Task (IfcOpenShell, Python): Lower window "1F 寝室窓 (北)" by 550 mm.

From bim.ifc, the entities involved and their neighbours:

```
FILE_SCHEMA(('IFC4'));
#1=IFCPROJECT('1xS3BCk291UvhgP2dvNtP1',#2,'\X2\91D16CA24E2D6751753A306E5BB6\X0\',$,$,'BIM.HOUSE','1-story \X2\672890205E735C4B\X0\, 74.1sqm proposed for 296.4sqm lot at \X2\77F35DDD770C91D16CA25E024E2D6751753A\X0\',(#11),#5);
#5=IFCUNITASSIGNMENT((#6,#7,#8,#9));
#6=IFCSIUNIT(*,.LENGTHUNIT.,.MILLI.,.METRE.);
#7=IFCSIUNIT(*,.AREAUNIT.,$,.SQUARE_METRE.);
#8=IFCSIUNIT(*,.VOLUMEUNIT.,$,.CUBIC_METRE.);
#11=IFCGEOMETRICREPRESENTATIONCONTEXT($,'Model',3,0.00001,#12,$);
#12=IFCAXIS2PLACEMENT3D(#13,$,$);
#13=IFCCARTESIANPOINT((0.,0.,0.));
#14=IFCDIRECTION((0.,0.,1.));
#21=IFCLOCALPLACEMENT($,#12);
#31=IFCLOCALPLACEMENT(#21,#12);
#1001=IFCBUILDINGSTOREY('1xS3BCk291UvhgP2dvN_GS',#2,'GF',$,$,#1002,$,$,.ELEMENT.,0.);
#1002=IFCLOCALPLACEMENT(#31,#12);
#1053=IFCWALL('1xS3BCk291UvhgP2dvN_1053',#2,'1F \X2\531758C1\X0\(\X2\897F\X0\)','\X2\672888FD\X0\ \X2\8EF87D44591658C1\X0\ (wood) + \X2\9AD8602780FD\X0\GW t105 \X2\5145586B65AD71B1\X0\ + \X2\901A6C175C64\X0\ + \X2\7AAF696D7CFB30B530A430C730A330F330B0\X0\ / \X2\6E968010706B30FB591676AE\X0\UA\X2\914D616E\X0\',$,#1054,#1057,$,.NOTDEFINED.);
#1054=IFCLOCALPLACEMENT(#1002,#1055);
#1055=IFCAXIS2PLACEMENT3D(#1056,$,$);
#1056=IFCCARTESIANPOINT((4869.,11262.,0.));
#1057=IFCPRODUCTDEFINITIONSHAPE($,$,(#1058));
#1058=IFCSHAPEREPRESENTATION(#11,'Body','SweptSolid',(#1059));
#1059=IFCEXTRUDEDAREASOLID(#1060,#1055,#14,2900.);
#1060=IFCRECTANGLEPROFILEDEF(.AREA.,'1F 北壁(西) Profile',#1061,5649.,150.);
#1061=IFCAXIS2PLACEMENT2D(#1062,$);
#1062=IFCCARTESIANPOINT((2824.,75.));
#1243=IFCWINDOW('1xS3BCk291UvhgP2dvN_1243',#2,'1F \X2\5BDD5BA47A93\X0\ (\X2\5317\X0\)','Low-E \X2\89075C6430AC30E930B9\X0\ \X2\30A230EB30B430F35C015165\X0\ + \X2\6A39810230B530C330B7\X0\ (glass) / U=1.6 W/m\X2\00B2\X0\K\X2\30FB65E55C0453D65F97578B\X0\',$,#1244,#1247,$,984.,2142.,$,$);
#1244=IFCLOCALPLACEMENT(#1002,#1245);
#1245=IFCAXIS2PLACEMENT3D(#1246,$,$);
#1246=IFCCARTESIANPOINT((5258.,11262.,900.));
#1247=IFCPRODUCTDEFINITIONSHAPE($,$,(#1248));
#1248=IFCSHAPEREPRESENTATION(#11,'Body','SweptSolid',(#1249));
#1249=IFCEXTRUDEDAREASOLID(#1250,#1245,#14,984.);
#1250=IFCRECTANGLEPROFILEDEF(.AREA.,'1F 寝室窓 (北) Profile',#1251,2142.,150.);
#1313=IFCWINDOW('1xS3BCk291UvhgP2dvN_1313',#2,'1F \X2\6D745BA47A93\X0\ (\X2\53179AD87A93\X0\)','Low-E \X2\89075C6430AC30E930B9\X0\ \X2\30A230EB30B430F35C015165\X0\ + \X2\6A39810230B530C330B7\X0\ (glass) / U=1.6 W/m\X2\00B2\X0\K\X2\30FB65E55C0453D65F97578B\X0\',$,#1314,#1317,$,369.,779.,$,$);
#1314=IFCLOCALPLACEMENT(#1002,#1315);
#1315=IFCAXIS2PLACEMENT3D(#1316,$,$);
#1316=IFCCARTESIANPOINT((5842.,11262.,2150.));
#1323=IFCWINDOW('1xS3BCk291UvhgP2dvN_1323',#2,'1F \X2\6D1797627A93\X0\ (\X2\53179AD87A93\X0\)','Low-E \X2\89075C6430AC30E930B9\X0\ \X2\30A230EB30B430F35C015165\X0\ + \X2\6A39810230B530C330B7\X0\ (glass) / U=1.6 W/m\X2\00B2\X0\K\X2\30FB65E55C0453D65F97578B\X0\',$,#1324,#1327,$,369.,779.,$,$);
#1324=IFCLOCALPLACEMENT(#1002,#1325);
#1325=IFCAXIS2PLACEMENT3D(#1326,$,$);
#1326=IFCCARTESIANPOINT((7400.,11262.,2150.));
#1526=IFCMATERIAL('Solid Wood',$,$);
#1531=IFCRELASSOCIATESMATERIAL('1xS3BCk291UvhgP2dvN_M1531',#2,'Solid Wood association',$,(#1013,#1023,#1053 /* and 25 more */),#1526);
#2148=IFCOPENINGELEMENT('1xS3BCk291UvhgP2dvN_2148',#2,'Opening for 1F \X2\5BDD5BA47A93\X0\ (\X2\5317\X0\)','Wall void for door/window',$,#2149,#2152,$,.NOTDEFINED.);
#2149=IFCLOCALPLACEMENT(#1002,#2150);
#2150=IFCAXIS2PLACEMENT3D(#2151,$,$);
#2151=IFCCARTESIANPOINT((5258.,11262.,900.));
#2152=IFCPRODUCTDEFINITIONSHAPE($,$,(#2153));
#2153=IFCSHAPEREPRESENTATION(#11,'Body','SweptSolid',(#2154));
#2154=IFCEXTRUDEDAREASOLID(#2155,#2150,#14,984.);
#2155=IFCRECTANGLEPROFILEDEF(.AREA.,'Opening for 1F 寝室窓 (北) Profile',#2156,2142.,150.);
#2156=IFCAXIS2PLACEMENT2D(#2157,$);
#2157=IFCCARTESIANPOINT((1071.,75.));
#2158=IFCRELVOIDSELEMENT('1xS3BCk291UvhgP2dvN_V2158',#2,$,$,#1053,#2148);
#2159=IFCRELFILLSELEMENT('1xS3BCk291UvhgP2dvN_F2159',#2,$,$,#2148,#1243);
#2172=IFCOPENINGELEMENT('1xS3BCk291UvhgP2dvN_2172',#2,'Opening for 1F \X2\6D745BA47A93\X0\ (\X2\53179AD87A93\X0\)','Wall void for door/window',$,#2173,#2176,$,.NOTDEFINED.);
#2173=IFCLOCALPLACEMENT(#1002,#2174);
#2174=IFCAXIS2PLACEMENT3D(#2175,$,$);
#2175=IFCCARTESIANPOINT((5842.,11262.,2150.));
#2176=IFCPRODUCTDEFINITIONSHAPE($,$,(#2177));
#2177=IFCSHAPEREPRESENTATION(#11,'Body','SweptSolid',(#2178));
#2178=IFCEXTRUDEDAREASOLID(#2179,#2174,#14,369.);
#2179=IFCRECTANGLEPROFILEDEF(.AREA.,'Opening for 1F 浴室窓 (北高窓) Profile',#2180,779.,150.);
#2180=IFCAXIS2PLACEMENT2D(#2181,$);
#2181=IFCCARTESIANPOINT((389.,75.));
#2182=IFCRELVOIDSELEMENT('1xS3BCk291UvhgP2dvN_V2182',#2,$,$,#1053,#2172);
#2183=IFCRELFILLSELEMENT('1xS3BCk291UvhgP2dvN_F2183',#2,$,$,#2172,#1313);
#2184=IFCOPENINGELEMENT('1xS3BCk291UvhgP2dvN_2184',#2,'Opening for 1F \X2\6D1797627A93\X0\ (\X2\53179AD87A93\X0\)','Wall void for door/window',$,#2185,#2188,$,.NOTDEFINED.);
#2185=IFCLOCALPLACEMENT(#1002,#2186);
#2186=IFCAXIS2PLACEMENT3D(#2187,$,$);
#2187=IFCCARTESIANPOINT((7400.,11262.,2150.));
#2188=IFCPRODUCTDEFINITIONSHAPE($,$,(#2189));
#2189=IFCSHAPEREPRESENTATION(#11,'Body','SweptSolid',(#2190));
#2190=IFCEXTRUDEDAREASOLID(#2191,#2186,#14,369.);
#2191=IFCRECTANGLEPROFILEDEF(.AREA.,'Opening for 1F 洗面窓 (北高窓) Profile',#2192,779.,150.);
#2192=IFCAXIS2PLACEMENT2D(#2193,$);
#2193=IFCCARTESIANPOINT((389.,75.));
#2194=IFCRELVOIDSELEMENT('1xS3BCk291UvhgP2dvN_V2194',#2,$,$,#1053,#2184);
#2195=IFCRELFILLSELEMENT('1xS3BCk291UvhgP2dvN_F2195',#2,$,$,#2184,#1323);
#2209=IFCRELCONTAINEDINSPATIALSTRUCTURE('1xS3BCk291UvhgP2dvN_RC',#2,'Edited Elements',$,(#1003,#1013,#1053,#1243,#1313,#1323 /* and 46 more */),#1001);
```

```python
import numpy as np
import ifcopenshell
import ifcopenshell.api.geometry
import ifcopenshell.util.placement
import ifcopenshell.util.unit

model = ifcopenshell.open("bim.ifc")
unit_scale = ifcopenshell.util.unit.calculate_unit_scale(model)

window = model.by_id(1243)
opening = window.FillsVoids[0].RelatingOpeningElement
dz = -550.0

shift = np.array([0.0, 0.0, dz])
# The window is not placed relative to its opening, so move both.
for product in (opening, window):
    matrix = ifcopenshell.util.placement.get_local_placement(product.ObjectPlacement)
    matrix[:3, 3] += shift
    ifcopenshell.api.geometry.edit_object_placement(model, product=product, matrix=matrix, is_si=False)

print(f"moved by {dz * unit_scale:+.3f} m")

model.write("bim_edited.ifc")
```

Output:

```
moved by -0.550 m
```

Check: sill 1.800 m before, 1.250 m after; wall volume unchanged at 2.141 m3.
